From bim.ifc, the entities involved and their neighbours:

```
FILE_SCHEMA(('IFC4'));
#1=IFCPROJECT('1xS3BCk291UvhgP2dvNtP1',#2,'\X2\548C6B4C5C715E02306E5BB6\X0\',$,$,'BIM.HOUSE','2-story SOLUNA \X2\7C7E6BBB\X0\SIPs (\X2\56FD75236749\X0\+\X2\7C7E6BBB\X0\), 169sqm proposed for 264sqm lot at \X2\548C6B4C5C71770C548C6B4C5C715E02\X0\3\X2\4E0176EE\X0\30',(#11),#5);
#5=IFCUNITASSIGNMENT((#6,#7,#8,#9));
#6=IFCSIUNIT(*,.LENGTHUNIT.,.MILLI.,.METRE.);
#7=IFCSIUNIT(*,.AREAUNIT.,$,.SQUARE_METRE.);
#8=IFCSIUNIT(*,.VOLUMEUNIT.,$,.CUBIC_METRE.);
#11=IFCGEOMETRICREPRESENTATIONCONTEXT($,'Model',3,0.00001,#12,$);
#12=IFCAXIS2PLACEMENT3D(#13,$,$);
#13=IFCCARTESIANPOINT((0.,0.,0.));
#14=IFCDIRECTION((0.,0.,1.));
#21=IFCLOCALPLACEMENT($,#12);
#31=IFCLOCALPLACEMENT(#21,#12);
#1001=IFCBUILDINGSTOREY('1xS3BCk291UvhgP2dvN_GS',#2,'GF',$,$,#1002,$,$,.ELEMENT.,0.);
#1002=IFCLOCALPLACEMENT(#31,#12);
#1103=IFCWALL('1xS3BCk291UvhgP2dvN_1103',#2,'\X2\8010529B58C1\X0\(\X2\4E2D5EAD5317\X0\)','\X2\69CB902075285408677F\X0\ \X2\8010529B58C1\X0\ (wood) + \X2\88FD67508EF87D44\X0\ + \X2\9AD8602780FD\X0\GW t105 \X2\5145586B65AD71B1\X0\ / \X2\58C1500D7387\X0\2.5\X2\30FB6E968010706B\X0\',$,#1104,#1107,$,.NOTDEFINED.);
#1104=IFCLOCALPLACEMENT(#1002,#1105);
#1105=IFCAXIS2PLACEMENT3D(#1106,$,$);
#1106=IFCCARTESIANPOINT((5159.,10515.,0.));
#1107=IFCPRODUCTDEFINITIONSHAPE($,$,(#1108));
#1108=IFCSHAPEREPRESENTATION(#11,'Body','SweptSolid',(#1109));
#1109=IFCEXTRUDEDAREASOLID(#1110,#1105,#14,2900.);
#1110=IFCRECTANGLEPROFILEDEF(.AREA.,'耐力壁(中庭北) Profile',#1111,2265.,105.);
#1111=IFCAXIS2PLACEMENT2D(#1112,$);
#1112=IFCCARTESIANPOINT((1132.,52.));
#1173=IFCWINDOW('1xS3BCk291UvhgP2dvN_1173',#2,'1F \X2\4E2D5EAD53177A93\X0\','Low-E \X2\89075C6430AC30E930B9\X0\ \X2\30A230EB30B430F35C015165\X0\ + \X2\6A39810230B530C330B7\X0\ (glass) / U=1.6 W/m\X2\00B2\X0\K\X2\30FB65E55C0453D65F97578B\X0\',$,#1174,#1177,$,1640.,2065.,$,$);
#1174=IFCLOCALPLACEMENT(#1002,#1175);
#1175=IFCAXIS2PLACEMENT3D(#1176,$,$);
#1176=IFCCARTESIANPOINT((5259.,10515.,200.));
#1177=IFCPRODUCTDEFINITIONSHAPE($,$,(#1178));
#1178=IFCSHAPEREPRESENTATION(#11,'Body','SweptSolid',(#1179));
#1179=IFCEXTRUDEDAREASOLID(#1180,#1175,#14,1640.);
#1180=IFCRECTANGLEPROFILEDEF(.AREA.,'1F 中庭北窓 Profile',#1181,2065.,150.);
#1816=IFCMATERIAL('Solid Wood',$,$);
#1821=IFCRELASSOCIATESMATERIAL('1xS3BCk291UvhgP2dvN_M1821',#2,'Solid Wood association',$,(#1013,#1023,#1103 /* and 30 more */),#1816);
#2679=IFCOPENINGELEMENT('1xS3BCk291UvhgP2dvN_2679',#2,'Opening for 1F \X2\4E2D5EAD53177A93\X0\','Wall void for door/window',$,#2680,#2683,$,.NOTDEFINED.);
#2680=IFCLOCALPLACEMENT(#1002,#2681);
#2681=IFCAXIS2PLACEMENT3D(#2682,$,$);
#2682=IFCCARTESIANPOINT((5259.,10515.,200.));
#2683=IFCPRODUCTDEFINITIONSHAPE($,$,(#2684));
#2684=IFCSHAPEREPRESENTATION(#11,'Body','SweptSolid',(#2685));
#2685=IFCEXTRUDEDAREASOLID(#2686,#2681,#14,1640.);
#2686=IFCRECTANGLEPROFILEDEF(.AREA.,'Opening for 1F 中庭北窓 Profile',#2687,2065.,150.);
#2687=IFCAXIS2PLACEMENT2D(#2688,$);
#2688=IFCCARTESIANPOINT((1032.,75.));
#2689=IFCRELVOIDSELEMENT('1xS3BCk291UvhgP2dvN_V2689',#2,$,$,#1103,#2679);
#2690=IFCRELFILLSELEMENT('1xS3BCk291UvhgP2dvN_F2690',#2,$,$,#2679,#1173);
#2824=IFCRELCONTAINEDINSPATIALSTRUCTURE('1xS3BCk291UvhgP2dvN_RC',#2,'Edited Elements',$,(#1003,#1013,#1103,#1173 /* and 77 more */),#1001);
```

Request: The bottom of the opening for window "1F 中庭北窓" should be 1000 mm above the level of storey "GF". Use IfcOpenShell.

```python
import numpy as np
import ifcopenshell
import ifcopenshell.api.geometry
import ifcopenshell.geom
import ifcopenshell.util.element
import ifcopenshell.util.placement
import ifcopenshell.util.shape
import ifcopenshell.util.unit

model = ifcopenshell.open("bim.ifc")
unit_scale = ifcopenshell.util.unit.calculate_unit_scale(model)

window = model.by_id(1173)
opening = window.FillsVoids[0].RelatingOpeningElement
storey = ifcopenshell.util.element.get_container(window, ifc_class="IfcBuildingStorey")
level = ifcopenshell.util.placement.get_local_placement(storey.ObjectPlacement)[2, 3]

# The opening's origin need not be at the sill, so measure its lowest point.
shape = ifcopenshell.geom.create_shape(ifcopenshell.geom.settings(), opening)
bottom = ifcopenshell.util.shape.get_shape_bottom_elevation(shape, shape.geometry) / unit_scale
dz = level + 1 / unit_scale - bottom

shift = np.array([0.0, 0.0, dz])
# The window is not placed relative to its opening, so move both.
for product in (opening, window):
    matrix = ifcopenshell.util.placement.get_local_placement(product.ObjectPlacement)
    matrix[:3, 3] += shift
    ifcopenshell.api.geometry.edit_object_placement(model, product=product, matrix=matrix, is_si=False)

print(f"moved by {dz * unit_scale:+.3f} m")

model.write("bim-out.ifc")
```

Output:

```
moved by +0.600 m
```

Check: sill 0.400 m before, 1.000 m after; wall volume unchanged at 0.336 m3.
